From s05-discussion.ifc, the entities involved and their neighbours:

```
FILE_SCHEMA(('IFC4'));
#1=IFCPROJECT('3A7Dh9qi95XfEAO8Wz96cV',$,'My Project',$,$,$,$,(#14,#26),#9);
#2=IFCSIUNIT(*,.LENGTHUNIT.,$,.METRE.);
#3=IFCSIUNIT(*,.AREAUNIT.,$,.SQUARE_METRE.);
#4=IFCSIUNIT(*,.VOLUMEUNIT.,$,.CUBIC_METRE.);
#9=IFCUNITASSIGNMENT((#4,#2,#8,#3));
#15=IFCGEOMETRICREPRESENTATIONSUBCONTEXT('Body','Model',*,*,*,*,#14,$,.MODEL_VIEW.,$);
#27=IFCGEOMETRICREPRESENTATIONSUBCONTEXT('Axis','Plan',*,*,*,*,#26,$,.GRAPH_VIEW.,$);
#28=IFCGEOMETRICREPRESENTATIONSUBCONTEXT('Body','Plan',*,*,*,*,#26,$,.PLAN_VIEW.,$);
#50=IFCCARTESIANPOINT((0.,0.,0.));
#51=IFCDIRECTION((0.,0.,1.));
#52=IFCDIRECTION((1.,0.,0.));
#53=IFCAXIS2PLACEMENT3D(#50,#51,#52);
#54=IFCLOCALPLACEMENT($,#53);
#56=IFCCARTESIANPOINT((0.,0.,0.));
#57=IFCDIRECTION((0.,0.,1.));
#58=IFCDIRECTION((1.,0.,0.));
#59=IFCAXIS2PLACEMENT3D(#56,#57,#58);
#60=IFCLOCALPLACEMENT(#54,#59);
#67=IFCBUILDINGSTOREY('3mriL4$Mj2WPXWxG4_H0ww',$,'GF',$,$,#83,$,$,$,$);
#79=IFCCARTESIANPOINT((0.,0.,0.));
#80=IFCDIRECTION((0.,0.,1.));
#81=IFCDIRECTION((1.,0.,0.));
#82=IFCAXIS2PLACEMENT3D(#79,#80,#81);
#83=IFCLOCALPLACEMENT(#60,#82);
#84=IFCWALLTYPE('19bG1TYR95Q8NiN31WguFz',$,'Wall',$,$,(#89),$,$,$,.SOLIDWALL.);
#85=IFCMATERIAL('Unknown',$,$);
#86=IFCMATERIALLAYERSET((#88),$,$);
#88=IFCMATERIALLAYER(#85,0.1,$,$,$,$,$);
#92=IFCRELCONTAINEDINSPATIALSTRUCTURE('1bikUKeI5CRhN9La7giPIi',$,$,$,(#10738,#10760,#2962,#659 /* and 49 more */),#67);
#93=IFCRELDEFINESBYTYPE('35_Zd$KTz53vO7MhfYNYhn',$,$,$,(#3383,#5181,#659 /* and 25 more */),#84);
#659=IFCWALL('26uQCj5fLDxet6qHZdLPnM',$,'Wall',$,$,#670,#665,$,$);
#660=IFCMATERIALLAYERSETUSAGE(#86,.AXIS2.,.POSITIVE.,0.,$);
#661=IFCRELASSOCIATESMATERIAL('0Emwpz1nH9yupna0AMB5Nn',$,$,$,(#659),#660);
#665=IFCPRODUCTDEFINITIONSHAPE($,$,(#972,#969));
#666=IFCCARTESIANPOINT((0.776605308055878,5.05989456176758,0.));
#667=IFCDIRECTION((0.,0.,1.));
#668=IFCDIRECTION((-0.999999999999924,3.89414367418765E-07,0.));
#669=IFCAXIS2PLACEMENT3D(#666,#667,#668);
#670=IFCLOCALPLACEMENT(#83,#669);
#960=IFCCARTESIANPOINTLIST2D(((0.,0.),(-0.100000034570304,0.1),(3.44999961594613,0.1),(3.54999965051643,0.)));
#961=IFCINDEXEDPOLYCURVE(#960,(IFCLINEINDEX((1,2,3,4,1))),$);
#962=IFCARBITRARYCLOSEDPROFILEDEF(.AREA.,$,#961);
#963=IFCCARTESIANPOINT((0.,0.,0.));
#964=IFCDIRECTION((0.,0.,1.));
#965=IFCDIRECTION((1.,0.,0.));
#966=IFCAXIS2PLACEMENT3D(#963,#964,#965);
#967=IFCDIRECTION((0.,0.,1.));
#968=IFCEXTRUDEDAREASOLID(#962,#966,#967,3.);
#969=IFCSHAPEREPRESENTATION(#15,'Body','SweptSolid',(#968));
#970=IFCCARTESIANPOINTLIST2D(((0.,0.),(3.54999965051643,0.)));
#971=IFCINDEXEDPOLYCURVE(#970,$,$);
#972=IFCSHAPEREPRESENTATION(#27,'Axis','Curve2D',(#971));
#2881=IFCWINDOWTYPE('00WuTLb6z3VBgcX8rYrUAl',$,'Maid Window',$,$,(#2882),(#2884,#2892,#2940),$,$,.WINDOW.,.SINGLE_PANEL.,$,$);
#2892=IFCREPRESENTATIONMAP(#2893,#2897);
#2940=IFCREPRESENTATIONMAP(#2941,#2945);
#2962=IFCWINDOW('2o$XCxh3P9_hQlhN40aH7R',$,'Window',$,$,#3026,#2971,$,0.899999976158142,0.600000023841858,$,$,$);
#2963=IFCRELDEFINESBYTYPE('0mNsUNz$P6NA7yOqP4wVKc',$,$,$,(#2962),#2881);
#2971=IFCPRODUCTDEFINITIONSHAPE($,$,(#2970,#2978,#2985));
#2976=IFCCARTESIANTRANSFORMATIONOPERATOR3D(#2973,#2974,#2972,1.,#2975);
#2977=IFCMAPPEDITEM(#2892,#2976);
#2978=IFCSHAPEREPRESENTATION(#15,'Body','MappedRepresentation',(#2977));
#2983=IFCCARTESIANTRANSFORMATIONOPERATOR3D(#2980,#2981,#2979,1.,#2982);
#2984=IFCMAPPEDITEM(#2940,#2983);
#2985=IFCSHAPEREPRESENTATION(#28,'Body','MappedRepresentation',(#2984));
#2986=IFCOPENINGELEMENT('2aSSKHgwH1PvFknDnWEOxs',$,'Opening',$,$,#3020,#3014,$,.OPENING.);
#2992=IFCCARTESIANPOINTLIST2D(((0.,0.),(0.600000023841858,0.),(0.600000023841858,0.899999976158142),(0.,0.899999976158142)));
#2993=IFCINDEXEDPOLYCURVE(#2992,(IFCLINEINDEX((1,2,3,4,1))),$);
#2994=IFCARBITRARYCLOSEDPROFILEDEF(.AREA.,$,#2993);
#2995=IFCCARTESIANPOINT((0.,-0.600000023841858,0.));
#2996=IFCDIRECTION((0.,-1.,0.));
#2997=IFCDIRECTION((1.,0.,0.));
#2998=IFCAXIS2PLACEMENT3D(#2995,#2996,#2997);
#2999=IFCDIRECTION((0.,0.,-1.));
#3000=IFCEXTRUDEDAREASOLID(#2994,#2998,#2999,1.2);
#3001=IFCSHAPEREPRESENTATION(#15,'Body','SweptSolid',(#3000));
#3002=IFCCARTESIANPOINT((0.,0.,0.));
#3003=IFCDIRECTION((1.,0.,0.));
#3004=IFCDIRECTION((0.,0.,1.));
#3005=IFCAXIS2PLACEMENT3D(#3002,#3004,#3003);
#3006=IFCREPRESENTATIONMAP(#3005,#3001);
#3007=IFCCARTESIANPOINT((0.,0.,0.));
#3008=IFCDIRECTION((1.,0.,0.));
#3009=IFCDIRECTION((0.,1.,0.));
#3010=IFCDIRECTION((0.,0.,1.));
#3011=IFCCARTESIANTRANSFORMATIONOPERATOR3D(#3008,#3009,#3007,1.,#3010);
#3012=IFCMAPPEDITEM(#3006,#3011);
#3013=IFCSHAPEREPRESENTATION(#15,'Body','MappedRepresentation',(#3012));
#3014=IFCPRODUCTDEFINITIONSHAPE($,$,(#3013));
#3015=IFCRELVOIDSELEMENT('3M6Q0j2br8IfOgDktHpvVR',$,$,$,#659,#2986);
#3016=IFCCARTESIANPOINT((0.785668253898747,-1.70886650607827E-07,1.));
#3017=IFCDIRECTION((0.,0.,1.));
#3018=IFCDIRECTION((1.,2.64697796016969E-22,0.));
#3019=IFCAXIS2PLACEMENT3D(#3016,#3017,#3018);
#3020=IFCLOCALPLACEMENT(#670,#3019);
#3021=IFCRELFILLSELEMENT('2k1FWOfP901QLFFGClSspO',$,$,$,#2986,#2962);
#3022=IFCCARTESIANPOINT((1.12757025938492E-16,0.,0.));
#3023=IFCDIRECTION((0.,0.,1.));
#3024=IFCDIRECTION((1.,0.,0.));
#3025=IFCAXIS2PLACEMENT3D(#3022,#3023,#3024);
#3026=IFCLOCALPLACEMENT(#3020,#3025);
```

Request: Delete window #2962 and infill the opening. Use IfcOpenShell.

```python
import ifcopenshell
import ifcopenshell.api.feature
import ifcopenshell.api.root
import ifcopenshell.geom
import ifcopenshell.util.shape

model = ifcopenshell.open("s05-discussion.ifc")
settings = ifcopenshell.geom.settings()


def volume(element):
    """Net volume in cubic metres, openings subtracted."""
    shape = ifcopenshell.geom.create_shape(settings, element)
    return ifcopenshell.util.shape.get_volume(shape.geometry)


window = model.by_guid("2o$XCxh3P9_hQlhN40aH7R")
opening = window.FillsVoids[0].RelatingOpeningElement
wall = opening.VoidsElements[0].RelatingBuildingElement
before = volume(wall)

ifcopenshell.api.root.remove_product(model, product=window)
ifcopenshell.api.feature.remove_feature(model, feature=opening)

after = volume(wall)

print(f"wall volume {before:.3f} -> {after:.3f} m3")

model.write("s05-discussion_rev.ifc")
```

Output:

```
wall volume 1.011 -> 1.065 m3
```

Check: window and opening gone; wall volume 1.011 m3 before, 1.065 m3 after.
